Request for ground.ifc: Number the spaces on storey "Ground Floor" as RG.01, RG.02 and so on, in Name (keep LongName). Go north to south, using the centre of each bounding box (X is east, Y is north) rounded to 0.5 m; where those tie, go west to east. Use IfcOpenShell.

First a look at what the model holds.

```python
import ifcopenshell
import ifcopenshell.util.element
import ifcopenshell.util.placement

model = ifcopenshell.open("ground.ifc")
print(model.schema)
storey = next(s for s in model.by_type("IfcBuildingStorey") if s.Name == "Ground Floor")
spaces = [e for e in ifcopenshell.util.element.get_decomposition(storey) if e.is_a("IfcSpace")]
for e in sorted(spaces, key=lambda e: e.id()):
    origin = ifcopenshell.util.placement.get_local_placement(e.ObjectPlacement)[:3, 3]
    print(e.id(), e.Name, e.LongName, origin.round(2) + 0.0, sep=" | ")
```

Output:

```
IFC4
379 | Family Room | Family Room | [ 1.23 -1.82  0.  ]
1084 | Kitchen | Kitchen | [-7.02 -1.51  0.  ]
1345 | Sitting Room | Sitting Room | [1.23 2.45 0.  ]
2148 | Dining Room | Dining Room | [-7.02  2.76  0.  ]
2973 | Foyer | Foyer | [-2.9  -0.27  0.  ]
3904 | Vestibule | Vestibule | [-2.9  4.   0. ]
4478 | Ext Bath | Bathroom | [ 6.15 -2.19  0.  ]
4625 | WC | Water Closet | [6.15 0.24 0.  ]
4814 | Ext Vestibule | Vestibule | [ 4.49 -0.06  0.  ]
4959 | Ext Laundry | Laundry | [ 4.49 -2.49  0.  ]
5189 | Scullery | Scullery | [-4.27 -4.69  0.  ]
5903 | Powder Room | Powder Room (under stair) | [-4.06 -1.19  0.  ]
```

```python
import ifcopenshell
import ifcopenshell.geom
import ifcopenshell.util.element
import ifcopenshell.util.shape

model = ifcopenshell.open("ground.ifc")
settings = ifcopenshell.geom.settings()
settings.set("use-world-coords", True)


def centre(element):
    shape = ifcopenshell.geom.create_shape(settings, element)
    return ifcopenshell.util.shape.get_bbox_centroid(shape.geometry)


storey = next(s for s in model.by_type("IfcBuildingStorey") if s.Name == "Ground Floor")
spaces = [e for e in ifcopenshell.util.element.get_decomposition(storey) if e.is_a("IfcSpace")]

# Insertion points can sit at a corner or the storey origin, so sort by the geometry (in metres).
centres = {e: centre(e) for e in spaces}
spaces.sort(key=lambda e: (-round(centres[e][1] / 0.5), centres[e][0]))

for i, e in enumerate(spaces, start=1):
    number = f"RG.{i:02d}"
    e.Name = number
    print(e.id(), number)

model.write("ground_rev.ifc")
```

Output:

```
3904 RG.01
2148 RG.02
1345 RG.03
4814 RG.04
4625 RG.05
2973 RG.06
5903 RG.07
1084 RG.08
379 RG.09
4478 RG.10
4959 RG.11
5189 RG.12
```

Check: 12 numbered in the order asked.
